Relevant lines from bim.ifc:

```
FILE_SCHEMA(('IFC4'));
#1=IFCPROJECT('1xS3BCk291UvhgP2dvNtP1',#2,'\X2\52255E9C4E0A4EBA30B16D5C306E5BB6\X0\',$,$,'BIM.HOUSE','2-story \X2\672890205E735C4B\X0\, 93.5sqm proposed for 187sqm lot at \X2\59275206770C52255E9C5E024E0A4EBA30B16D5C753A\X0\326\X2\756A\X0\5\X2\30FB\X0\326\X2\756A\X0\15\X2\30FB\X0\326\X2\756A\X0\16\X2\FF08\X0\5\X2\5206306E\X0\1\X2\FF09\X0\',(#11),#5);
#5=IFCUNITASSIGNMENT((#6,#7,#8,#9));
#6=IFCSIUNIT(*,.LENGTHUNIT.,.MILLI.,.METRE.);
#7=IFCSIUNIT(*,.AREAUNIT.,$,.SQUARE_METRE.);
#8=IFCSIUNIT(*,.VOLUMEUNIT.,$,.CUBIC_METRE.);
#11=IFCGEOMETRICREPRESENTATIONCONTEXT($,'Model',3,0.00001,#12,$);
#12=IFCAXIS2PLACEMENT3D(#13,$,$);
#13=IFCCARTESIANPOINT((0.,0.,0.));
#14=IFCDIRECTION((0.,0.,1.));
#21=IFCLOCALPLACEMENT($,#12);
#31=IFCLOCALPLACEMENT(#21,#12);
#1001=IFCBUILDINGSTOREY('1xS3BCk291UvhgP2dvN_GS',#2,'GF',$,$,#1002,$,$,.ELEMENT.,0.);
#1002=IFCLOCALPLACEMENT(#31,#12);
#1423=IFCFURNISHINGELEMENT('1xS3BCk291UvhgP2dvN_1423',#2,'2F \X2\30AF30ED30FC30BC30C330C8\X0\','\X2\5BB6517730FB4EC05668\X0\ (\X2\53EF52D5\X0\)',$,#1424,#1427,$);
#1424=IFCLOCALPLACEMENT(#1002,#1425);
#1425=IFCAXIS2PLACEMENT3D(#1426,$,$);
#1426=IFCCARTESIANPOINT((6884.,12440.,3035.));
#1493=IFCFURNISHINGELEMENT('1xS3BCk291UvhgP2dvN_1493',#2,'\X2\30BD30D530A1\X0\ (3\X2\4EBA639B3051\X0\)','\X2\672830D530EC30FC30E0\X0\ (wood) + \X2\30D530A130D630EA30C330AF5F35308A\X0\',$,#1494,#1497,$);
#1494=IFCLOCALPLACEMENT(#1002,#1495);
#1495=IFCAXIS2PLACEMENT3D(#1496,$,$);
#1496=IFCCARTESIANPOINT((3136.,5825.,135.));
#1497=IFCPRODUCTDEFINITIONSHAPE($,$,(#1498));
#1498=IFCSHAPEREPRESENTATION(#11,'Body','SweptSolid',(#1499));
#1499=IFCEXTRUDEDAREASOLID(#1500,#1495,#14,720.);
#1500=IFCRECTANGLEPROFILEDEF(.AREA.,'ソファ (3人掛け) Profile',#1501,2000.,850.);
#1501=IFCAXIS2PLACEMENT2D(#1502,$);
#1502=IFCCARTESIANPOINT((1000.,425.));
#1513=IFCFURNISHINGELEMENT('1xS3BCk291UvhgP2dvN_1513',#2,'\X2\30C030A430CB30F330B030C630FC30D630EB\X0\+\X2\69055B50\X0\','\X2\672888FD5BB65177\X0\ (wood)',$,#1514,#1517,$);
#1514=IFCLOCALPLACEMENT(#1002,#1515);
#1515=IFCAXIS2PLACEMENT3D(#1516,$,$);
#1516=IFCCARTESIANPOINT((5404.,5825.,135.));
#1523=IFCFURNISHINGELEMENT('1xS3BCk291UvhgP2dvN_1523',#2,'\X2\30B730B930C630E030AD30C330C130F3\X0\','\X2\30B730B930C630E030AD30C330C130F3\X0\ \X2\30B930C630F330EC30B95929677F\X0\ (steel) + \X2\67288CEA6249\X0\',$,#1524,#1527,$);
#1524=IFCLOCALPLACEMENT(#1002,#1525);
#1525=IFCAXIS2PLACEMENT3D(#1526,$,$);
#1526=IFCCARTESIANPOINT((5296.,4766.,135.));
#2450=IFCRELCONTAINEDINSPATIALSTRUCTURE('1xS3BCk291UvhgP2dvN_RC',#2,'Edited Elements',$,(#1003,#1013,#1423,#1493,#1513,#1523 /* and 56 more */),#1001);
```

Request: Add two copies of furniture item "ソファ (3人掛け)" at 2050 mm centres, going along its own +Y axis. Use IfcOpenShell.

```python
import ifcopenshell
import ifcopenshell.api.geometry
import ifcopenshell.api.root
import ifcopenshell.util.element
import ifcopenshell.util.placement

model = ifcopenshell.open("bim.ifc")


def reuse_history(source, copy):
    """copy_class also copies each property set's owner history, people and application; keep the originals."""
    for rel in copy.IsDefinedBy:
        if rel.is_a("IfcRelDefinesByProperties") and (history := rel.RelatingPropertyDefinition.OwnerHistory):
            rel.RelatingPropertyDefinition.OwnerHistory = source.OwnerHistory
            ifcopenshell.util.element.remove_deep2(model, history)


source = model.by_id(1493)
base = ifcopenshell.util.placement.get_local_placement(source.ObjectPlacement)
step = base[:3, 1] * 2050.0

for i in range(1, 3):
    copy = ifcopenshell.api.root.copy_class(model, product=source)
    copy.Representation = ifcopenshell.util.element.copy_deep(
        model, source.Representation, exclude=["IfcGeometricRepresentationContext", "IfcRepresentationMap"]
    )
    reuse_history(source, copy)
    matrix = base.copy()
    matrix[:3, 3] += i * step
    print("added at", matrix[:3, 3].round(3) + 0.0)
    ifcopenshell.api.geometry.edit_object_placement(model, product=copy, matrix=matrix, is_si=False)

model.write("bim_rev.ifc")
```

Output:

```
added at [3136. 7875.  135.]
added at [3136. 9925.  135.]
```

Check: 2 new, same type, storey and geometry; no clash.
